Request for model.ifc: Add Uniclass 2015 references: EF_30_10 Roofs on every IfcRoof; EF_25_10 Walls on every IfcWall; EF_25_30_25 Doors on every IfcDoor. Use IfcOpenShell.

First a look at what the model holds.

```python
import ifcopenshell

model = ifcopenshell.open("model.ifc")
print(model.schema)
print("classifications:", [c.Name for c in model.by_type("IfcClassification")])
for ifc_class in ("IfcDoor", "IfcRoof", "IfcStair", "IfcWall", "IfcWindow"):
    print(ifc_class, len(model.by_type(ifc_class)))
```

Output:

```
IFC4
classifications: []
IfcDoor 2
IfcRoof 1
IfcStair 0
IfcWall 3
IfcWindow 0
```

```python
import ifcopenshell
import ifcopenshell.api.classification

model = ifcopenshell.open("model.ifc")

system = ifcopenshell.api.classification.add_classification(model, classification="Uniclass 2015")

codes = {
    "IfcRoof": ("EF_30_10", "Roofs"),
    "IfcWall": ("EF_25_10", "Walls"),
    "IfcDoor": ("EF_25_30_25", "Doors"),
}
for ifc_class, (code, name) in codes.items():
    products = model.by_type(ifc_class)
    ifcopenshell.api.classification.add_reference(
        model, products=products, classification=system, identification=code, name=name
    )
    print(code, len(products))

model.write("model_rev.ifc")
```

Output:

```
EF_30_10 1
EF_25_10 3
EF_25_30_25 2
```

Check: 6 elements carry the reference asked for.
